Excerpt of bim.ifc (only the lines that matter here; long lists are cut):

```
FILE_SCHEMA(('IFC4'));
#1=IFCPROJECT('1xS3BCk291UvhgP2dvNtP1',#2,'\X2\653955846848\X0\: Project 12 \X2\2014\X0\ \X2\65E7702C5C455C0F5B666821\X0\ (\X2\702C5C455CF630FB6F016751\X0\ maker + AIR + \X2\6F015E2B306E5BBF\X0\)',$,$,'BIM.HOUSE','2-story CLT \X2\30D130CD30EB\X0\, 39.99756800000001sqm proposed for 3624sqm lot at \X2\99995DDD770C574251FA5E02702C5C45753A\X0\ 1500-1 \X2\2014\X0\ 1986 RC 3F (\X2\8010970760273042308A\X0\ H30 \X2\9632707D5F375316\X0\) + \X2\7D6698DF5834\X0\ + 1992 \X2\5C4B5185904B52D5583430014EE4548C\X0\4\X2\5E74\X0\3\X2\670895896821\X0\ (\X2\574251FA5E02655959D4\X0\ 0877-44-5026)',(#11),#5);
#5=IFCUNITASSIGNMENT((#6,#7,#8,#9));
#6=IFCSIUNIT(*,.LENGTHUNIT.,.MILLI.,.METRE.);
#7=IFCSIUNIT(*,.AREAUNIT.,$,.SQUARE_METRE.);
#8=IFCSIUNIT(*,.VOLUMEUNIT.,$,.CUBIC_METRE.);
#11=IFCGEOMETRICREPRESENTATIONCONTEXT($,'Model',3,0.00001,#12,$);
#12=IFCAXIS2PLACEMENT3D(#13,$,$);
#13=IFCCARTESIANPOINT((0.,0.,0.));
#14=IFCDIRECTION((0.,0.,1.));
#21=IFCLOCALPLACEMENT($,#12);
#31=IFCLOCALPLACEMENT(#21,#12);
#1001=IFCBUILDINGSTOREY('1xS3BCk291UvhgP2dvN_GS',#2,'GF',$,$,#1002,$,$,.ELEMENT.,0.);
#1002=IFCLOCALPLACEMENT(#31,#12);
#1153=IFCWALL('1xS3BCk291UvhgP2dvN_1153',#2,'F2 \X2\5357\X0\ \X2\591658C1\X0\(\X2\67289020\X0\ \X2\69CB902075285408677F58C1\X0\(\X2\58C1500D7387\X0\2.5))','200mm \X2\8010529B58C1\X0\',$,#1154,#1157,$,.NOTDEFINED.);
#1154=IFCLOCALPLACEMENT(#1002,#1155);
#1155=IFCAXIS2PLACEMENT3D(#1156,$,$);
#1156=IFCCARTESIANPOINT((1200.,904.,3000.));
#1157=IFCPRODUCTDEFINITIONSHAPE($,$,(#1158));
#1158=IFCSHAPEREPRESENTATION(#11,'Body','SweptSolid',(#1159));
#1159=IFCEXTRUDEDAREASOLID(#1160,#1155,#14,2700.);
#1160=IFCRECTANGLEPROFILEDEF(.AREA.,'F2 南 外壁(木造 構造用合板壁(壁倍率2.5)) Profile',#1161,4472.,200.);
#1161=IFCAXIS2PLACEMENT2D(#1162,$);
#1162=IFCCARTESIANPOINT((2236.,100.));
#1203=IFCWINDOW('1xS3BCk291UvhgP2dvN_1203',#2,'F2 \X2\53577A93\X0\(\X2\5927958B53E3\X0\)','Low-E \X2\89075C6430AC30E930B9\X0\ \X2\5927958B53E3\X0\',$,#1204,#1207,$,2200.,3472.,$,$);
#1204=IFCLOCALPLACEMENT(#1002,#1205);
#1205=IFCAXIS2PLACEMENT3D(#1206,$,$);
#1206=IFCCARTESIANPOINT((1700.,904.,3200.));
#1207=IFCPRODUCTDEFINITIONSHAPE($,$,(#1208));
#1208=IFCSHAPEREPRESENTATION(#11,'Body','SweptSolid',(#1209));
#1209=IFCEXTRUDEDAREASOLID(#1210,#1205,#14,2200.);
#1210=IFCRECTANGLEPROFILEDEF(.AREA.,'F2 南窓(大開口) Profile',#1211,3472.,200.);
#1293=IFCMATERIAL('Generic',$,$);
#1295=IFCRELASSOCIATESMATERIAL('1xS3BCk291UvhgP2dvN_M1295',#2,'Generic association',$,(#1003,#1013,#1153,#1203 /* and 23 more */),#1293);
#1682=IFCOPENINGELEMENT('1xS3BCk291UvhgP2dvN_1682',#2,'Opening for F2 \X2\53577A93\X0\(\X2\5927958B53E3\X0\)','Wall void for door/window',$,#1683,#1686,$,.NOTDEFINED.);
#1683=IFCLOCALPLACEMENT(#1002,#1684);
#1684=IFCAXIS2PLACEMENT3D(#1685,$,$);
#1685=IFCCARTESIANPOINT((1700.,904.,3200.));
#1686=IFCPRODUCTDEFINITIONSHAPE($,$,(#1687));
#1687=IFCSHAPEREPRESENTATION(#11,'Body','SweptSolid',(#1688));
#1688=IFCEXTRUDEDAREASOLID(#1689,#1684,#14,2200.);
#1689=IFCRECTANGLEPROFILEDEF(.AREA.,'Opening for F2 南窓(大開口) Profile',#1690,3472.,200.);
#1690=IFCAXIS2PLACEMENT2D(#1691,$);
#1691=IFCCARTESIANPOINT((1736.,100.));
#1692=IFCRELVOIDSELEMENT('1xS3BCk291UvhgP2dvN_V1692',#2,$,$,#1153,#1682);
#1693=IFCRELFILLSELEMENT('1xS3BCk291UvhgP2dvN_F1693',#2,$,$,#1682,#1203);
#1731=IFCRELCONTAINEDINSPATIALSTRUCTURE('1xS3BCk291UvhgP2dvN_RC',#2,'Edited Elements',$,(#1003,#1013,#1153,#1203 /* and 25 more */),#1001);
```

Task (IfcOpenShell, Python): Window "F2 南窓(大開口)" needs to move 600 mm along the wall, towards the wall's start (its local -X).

```python
import ifcopenshell
import ifcopenshell.api.geometry
import ifcopenshell.util.placement
import ifcopenshell.util.unit

model = ifcopenshell.open("bim.ifc")
unit_scale = ifcopenshell.util.unit.calculate_unit_scale(model)

window = model.by_id(1203)
opening = window.FillsVoids[0].RelatingOpeningElement
wall = opening.VoidsElements[0].RelatingBuildingElement

wall_matrix = ifcopenshell.util.placement.get_local_placement(wall.ObjectPlacement)
shift = wall_matrix[:3, 0] * -0.6 / unit_scale
before = ifcopenshell.util.placement.get_local_placement(window.ObjectPlacement)[:3, 3].copy()

# The window is not placed relative to its opening, so move both.
for product in (opening, window):
    matrix = ifcopenshell.util.placement.get_local_placement(product.ObjectPlacement)
    matrix[:3, 3] += shift
    ifcopenshell.api.geometry.edit_object_placement(model, product=product, matrix=matrix, is_si=False)

after = ifcopenshell.util.placement.get_local_placement(window.ObjectPlacement)[:3, 3]
print("window moved by", (after - before).round(3) + 0.0)

model.write("bim_v2.ifc")
```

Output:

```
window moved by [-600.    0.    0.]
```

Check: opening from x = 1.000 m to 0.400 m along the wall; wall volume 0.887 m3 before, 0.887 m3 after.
